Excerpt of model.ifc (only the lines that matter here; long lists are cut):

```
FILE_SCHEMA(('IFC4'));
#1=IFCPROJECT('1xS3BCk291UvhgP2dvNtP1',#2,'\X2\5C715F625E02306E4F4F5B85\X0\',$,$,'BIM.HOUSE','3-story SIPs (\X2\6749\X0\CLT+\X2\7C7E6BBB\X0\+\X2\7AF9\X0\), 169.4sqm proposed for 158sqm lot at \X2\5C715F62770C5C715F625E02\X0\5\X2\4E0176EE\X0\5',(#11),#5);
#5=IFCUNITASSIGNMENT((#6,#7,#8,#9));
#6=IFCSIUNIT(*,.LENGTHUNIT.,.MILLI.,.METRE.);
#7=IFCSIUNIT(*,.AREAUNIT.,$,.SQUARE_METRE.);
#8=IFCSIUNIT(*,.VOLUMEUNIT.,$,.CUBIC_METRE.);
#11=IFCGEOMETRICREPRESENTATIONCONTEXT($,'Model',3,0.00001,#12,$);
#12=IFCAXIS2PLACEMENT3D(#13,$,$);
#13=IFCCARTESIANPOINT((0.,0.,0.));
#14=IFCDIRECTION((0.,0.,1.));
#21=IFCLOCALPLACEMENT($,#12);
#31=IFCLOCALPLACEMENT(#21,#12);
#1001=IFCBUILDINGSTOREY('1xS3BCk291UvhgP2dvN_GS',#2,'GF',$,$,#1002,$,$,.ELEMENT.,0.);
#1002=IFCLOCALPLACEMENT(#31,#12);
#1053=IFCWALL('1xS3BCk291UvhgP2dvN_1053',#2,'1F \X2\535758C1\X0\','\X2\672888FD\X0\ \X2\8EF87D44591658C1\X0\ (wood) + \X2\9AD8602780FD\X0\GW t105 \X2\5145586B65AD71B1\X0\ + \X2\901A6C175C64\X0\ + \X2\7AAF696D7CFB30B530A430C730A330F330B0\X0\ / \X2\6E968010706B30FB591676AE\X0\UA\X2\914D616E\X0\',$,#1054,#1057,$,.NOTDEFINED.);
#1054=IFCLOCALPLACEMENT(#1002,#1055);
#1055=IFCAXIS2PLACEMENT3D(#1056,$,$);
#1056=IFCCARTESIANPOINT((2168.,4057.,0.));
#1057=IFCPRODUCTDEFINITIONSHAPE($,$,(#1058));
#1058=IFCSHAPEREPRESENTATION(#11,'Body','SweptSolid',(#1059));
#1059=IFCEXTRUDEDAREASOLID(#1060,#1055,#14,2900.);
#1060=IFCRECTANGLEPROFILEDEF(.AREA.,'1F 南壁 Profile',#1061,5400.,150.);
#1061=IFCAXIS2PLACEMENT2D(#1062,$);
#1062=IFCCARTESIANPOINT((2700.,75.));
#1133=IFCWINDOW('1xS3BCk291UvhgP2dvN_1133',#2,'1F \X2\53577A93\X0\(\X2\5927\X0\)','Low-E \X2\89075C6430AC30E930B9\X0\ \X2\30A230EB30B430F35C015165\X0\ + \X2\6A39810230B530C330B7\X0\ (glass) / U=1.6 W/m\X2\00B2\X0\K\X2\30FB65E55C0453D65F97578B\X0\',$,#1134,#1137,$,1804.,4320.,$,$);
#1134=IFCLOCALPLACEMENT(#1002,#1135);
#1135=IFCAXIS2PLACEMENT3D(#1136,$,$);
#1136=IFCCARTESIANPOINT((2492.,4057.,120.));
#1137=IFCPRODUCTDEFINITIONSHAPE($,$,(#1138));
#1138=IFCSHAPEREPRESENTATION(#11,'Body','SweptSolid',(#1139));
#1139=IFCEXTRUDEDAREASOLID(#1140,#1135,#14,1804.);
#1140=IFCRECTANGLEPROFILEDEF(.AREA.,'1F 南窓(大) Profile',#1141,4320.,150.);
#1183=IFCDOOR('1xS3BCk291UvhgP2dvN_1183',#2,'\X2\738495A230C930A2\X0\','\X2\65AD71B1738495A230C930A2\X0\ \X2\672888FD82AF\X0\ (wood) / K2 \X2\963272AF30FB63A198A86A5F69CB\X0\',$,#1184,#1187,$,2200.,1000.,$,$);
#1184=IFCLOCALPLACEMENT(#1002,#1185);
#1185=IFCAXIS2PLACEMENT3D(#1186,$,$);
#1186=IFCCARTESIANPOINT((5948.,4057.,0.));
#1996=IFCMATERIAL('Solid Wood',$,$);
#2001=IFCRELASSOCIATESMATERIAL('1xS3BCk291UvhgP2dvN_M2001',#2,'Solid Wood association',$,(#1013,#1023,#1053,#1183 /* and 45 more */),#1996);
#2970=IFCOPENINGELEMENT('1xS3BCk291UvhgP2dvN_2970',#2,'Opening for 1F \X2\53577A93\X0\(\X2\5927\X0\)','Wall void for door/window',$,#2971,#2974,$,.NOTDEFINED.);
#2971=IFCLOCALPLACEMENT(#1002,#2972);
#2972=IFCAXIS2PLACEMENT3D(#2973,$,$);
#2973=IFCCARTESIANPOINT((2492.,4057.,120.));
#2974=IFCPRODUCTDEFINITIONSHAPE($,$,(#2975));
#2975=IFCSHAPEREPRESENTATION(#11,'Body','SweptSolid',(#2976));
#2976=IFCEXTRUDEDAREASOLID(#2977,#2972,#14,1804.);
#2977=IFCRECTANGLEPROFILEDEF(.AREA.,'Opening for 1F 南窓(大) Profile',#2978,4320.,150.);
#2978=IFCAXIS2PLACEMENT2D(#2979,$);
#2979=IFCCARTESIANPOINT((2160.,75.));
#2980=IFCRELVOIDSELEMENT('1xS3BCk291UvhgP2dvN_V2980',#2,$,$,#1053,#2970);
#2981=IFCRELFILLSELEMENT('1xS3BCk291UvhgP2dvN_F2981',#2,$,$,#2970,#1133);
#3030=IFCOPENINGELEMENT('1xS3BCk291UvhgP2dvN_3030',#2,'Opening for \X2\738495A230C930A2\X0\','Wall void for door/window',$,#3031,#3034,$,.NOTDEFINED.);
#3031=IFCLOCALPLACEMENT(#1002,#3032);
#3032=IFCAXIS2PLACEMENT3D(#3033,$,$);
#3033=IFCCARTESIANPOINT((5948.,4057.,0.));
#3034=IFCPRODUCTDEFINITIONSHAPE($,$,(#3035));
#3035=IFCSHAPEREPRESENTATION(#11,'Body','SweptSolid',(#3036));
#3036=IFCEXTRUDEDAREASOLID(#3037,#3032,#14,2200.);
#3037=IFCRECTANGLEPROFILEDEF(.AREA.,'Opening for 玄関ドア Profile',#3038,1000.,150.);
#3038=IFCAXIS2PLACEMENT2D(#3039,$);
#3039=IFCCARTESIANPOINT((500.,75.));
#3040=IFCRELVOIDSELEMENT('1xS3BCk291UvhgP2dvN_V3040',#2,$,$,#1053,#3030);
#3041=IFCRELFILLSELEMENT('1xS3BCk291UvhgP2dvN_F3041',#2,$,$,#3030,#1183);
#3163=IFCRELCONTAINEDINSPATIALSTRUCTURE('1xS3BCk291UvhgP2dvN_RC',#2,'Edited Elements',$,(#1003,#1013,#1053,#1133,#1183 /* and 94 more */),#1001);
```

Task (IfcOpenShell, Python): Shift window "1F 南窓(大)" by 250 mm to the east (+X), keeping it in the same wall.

```python
import ifcopenshell
import ifcopenshell.api.geometry
import ifcopenshell.util.placement

model = ifcopenshell.open("model.ifc")

window = model.by_id(1133)
opening = window.FillsVoids[0].RelatingOpeningElement
wall = opening.VoidsElements[0].RelatingBuildingElement

wall_matrix = ifcopenshell.util.placement.get_local_placement(wall.ObjectPlacement)
shift = wall_matrix[:3, 0] * 250.0
before = ifcopenshell.util.placement.get_local_placement(window.ObjectPlacement)[:3, 3].copy()

# The window is not placed relative to its opening, so move both.
for product in (opening, window):
    matrix = ifcopenshell.util.placement.get_local_placement(product.ObjectPlacement)
    matrix[:3, 3] += shift
    ifcopenshell.api.geometry.edit_object_placement(model, product=product, matrix=matrix, is_si=False)

after = ifcopenshell.util.placement.get_local_placement(window.ObjectPlacement)[:3, 3]
print("window moved by", (after - before).round(3) + 0.0)

model.write("model_rev.ifc")
```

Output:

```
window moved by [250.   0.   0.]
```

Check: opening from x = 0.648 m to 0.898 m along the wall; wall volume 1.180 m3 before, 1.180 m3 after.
